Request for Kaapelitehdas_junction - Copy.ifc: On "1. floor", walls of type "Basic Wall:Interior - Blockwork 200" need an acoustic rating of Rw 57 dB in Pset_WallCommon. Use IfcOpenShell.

First a look at what the model holds.

```python
import ifcopenshell
import ifcopenshell.util.element

model = ifcopenshell.open("Kaapelitehdas_junction - Copy.ifc")
print(model.schema)
storey = next(s for s in model.by_type("IfcBuildingStorey") if s.Name == "1. floor")
walls = [e for e in ifcopenshell.util.element.get_decomposition(storey) if e.is_a("IfcWall")]
seen = {}
for e in walls:
    element_type = ifcopenshell.util.element.get_type(e)
    key = (element_type.Name if element_type != e and element_type else None, ifcopenshell.util.element.get_pset(e, "Pset_WallCommon", "AcousticRating"))
    seen[key] = seen.get(key, 0) + 1
for (name, value), count in sorted(seen.items(), key=str):
    print(count, "x", name, "|", value)
```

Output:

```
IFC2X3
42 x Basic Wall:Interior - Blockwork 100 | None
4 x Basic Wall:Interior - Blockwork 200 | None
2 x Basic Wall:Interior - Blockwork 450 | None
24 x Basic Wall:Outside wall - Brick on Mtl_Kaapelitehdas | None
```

```python
import ifcopenshell
import ifcopenshell.api.pset
import ifcopenshell.util.element

model = ifcopenshell.open("Kaapelitehdas_junction - Copy.ifc")

storey = next(s for s in model.by_type("IfcBuildingStorey") if s.Name == "1. floor")
walls = [e for e in ifcopenshell.util.element.get_decomposition(storey) if e.is_a("IfcWall")]

count = 0
for e in walls:
    element_type = ifcopenshell.util.element.get_type(e)
    if element_type in (None, e) or element_type.Name != "Basic Wall:Interior - Blockwork 200":
        continue
    # add_pset returns the element's existing set when there is one.
    pset = ifcopenshell.api.pset.add_pset(model, product=e, name="Pset_WallCommon")
    ifcopenshell.api.pset.edit_pset(model, pset=pset, properties={"AcousticRating": "Rw 57 dB"})
    count += 1

print(count, "walls updated")

model.write("Kaapelitehdas_junction - Copy_v2.ifc")
```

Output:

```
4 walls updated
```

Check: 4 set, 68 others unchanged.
